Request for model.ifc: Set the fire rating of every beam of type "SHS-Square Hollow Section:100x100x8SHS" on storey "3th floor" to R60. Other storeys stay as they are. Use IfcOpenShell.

First a look at what the model holds.

```python
import ifcopenshell
import ifcopenshell.util.element

model = ifcopenshell.open("model.ifc")
print(model.schema)
storey = next(s for s in model.by_type("IfcBuildingStorey") if s.Name == "3th floor")
beams = [e for e in ifcopenshell.util.element.get_decomposition(storey) if e.is_a("IfcBeam")]
seen = {}
for e in beams:
    element_type = ifcopenshell.util.element.get_type(e)
    key = (element_type.Name if element_type != e and element_type else None, ifcopenshell.util.element.get_pset(e, "Pset_BeamCommon", "FireRating"))
    seen[key] = seen.get(key, 0) + 1
for (name, value), count in sorted(seen.items(), key=str):
    print(count, "x", name, "|", value)
```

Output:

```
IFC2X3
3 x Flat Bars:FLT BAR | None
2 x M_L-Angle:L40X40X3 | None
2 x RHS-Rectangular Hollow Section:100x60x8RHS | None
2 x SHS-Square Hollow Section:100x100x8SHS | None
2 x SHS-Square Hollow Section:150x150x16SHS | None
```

```python
import ifcopenshell
import ifcopenshell.api.pset
import ifcopenshell.util.element

model = ifcopenshell.open("model.ifc")

storey = next(s for s in model.by_type("IfcBuildingStorey") if s.Name == "3th floor")
beams = [e for e in ifcopenshell.util.element.get_decomposition(storey) if e.is_a("IfcBeam")]

count = 0
for e in beams:
    element_type = ifcopenshell.util.element.get_type(e)
    if element_type in (None, e) or element_type.Name != "SHS-Square Hollow Section:100x100x8SHS":
        continue
    # add_pset returns the element's existing set when there is one.
    pset = ifcopenshell.api.pset.add_pset(model, product=e, name="Pset_BeamCommon")
    ifcopenshell.api.pset.edit_pset(model, pset=pset, properties={"FireRating": "R60"})
    count += 1

print(count, "beams updated")

model.write("model_rev.ifc")
```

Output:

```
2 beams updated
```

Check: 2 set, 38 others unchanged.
